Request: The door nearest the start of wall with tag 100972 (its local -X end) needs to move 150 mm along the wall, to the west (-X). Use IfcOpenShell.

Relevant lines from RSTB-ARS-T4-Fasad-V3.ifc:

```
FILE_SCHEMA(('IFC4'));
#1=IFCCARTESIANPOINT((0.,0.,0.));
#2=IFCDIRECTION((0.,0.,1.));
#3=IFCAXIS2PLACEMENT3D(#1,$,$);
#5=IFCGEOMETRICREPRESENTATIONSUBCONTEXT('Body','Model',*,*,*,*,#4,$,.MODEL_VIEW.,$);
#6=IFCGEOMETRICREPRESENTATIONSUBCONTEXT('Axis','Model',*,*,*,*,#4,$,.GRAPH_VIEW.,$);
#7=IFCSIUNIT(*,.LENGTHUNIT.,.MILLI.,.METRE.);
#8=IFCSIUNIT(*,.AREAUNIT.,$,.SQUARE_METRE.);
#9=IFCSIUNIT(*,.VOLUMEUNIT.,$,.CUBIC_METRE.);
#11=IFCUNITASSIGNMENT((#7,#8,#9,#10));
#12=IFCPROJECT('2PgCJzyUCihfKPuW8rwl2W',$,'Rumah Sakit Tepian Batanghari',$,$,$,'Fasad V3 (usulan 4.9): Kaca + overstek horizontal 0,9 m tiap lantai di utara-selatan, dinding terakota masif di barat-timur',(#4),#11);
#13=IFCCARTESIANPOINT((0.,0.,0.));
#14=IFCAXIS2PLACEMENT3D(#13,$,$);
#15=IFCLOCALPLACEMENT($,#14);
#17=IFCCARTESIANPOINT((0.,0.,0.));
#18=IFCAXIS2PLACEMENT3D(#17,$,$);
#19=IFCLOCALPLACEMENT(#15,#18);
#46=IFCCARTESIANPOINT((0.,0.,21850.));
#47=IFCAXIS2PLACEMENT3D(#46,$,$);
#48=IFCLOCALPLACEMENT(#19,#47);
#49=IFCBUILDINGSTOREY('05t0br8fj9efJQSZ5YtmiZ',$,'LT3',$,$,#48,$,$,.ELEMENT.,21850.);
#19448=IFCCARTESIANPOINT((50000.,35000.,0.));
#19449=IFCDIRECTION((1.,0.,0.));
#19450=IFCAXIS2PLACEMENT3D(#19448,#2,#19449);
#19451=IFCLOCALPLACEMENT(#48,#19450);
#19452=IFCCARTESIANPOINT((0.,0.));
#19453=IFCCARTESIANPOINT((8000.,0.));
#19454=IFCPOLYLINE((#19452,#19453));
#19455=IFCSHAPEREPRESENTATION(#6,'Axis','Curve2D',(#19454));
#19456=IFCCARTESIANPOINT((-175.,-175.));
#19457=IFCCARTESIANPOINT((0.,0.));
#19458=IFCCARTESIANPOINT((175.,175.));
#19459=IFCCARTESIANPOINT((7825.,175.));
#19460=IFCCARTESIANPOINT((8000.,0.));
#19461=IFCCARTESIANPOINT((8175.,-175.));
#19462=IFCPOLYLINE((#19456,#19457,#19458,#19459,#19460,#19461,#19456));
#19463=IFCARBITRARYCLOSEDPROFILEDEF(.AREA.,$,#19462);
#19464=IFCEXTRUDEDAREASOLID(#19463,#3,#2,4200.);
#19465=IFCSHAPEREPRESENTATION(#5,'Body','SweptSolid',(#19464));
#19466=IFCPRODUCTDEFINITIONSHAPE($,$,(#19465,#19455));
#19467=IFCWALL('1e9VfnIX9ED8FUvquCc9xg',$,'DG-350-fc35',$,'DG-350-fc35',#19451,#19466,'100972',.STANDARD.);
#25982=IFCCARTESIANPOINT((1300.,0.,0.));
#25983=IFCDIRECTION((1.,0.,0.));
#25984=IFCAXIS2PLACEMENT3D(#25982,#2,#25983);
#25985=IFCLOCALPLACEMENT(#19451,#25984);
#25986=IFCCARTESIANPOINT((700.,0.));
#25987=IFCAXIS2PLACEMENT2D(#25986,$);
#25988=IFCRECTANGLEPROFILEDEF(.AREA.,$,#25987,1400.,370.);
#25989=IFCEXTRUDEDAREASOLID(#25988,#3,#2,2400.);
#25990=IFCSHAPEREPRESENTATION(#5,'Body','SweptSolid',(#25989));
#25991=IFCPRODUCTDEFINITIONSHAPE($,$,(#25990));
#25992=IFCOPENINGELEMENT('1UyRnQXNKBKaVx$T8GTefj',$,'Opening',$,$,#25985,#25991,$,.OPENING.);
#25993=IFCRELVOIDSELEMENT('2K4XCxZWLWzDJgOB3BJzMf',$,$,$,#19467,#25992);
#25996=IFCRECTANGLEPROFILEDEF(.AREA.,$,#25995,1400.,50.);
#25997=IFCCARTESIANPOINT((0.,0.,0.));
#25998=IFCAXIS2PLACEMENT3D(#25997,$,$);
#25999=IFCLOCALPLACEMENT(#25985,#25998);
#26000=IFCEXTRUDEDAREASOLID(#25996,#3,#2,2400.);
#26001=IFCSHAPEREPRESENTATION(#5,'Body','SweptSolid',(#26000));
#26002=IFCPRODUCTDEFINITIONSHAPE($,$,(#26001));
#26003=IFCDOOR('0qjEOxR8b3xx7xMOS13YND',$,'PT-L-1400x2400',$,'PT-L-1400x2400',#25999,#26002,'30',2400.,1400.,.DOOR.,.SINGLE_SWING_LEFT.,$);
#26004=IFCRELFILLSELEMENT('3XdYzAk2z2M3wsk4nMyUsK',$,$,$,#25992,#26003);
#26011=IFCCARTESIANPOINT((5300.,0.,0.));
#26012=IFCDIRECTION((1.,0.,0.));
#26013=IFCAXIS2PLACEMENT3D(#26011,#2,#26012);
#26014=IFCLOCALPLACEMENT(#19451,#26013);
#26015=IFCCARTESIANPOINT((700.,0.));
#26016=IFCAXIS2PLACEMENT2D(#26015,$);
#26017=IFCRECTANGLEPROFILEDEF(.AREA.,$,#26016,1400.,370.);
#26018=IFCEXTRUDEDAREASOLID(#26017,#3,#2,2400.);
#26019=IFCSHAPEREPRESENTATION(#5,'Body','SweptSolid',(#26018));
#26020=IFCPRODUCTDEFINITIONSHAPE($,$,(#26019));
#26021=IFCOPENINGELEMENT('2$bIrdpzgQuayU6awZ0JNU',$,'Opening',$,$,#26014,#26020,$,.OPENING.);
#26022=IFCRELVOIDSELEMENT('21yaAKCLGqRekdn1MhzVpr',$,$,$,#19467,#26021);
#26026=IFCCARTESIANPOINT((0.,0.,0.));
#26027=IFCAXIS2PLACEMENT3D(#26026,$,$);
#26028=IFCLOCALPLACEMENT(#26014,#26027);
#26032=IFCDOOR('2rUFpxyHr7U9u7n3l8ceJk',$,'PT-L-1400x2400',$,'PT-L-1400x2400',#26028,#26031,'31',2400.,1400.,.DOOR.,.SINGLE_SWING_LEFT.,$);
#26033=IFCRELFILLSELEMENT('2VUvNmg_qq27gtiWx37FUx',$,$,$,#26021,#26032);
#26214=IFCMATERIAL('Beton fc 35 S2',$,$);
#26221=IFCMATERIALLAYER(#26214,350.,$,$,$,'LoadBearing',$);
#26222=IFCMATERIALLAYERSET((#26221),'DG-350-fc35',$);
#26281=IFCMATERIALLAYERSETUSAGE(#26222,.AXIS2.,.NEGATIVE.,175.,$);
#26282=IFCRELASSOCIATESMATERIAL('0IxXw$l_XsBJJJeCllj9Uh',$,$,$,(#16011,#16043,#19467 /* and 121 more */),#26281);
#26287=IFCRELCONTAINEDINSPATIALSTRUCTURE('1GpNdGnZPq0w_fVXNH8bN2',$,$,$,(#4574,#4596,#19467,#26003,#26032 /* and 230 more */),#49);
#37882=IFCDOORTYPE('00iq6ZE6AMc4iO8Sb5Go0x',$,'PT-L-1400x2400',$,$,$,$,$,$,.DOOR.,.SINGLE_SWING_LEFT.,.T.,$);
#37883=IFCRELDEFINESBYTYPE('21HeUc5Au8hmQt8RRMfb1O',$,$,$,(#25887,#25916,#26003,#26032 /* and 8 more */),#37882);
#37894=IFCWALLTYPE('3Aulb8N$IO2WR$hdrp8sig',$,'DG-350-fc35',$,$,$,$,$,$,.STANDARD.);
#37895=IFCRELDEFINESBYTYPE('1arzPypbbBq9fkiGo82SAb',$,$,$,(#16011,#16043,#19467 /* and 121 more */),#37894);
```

```python
import ifcopenshell
import ifcopenshell.api.geometry
import ifcopenshell.util.placement
import ifcopenshell.util.unit

model = ifcopenshell.open("RSTB-ARS-T4-Fasad-V3.ifc")
unit_scale = ifcopenshell.util.unit.calculate_unit_scale(model)

door = model.by_guid("0qjEOxR8b3xx7xMOS13YND")
opening = door.FillsVoids[0].RelatingOpeningElement
wall = opening.VoidsElements[0].RelatingBuildingElement

wall_matrix = ifcopenshell.util.placement.get_local_placement(wall.ObjectPlacement)
shift = wall_matrix[:3, 0] * -0.15 / unit_scale
before = ifcopenshell.util.placement.get_local_placement(door.ObjectPlacement)[:3, 3].copy()

# The door is placed relative to its opening, so it follows when the opening moves.
matrix = ifcopenshell.util.placement.get_local_placement(opening.ObjectPlacement)
matrix[:3, 3] += shift
ifcopenshell.api.geometry.edit_object_placement(
    model, product=opening, matrix=matrix, is_si=False, should_transform_children=True
)

after = ifcopenshell.util.placement.get_local_placement(door.ObjectPlacement)[:3, 3]
print("door moved by", (after - before).round(3) + 0.0)

model.write("RSTB-ARS-T4-Fasad-V3_v2.ifc")
```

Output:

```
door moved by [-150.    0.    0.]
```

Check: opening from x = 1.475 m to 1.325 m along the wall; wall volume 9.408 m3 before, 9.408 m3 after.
